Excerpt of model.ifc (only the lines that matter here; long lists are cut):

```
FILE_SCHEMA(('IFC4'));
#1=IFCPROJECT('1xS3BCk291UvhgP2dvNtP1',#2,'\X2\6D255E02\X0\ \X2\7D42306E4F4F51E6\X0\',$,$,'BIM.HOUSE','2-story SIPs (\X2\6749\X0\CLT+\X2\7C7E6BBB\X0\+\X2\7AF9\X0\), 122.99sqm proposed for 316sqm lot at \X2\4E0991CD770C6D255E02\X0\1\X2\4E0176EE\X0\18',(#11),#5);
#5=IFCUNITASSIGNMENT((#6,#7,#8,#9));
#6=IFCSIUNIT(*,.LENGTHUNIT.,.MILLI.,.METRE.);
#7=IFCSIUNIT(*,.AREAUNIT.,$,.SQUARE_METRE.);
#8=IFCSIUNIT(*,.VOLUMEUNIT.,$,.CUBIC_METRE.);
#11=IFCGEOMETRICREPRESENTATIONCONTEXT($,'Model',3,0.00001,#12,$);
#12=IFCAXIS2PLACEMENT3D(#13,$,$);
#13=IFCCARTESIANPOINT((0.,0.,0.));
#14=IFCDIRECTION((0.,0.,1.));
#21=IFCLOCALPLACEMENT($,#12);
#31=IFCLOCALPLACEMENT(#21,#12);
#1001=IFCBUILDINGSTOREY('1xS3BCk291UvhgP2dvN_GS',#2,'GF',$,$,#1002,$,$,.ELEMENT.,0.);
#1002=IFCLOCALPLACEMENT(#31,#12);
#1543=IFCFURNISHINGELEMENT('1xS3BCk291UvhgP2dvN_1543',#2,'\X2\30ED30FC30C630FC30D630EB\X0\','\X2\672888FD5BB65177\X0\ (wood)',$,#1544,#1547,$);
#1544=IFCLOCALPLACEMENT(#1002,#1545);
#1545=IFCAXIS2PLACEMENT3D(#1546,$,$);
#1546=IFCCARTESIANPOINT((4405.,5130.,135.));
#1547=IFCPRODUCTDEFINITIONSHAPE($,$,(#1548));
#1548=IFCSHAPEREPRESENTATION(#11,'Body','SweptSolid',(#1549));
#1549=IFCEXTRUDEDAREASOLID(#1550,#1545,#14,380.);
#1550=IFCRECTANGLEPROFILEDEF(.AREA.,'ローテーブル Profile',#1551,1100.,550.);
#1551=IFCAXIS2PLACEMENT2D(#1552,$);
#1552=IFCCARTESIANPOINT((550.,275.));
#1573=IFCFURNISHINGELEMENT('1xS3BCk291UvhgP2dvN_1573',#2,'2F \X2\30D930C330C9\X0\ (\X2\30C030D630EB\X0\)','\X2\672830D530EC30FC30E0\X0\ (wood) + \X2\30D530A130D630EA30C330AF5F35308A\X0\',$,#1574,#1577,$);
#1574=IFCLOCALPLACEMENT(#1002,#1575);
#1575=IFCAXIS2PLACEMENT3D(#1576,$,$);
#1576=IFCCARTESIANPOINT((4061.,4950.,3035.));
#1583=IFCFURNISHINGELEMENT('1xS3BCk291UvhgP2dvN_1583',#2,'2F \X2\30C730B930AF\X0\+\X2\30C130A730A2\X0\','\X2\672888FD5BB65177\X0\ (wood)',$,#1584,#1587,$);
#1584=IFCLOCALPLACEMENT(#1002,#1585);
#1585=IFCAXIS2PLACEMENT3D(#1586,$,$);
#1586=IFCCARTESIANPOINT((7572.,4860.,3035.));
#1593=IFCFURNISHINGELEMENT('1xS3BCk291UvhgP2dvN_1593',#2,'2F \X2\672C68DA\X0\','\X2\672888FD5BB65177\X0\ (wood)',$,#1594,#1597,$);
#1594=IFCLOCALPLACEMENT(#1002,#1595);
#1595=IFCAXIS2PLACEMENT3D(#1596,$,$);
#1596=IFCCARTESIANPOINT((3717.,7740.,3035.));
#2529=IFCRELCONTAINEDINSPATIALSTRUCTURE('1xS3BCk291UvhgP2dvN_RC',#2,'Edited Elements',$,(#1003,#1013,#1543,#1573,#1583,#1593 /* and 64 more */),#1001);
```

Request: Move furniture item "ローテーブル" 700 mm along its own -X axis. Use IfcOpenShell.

```python
import ifcopenshell
import ifcopenshell.api.geometry
import ifcopenshell.util.placement
import ifcopenshell.util.unit

model = ifcopenshell.open("model.ifc")
unit_scale = ifcopenshell.util.unit.calculate_unit_scale(model)

item = model.by_guid("1xS3BCk291UvhgP2dvN_1543")
matrix = ifcopenshell.util.placement.get_local_placement(item.ObjectPlacement)
matrix[:3, 3] -= matrix[:3, 0] * 0.7 / unit_scale
ifcopenshell.api.geometry.edit_object_placement(model, product=item, matrix=matrix, is_si=False)

print(ifcopenshell.util.placement.get_local_placement(item.ObjectPlacement).round(3) + 0.0)

model.write("model_rev.ifc")
```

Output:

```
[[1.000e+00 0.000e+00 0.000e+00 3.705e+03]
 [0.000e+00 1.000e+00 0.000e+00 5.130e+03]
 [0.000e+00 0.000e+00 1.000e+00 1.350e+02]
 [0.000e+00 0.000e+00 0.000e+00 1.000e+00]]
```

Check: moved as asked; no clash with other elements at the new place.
